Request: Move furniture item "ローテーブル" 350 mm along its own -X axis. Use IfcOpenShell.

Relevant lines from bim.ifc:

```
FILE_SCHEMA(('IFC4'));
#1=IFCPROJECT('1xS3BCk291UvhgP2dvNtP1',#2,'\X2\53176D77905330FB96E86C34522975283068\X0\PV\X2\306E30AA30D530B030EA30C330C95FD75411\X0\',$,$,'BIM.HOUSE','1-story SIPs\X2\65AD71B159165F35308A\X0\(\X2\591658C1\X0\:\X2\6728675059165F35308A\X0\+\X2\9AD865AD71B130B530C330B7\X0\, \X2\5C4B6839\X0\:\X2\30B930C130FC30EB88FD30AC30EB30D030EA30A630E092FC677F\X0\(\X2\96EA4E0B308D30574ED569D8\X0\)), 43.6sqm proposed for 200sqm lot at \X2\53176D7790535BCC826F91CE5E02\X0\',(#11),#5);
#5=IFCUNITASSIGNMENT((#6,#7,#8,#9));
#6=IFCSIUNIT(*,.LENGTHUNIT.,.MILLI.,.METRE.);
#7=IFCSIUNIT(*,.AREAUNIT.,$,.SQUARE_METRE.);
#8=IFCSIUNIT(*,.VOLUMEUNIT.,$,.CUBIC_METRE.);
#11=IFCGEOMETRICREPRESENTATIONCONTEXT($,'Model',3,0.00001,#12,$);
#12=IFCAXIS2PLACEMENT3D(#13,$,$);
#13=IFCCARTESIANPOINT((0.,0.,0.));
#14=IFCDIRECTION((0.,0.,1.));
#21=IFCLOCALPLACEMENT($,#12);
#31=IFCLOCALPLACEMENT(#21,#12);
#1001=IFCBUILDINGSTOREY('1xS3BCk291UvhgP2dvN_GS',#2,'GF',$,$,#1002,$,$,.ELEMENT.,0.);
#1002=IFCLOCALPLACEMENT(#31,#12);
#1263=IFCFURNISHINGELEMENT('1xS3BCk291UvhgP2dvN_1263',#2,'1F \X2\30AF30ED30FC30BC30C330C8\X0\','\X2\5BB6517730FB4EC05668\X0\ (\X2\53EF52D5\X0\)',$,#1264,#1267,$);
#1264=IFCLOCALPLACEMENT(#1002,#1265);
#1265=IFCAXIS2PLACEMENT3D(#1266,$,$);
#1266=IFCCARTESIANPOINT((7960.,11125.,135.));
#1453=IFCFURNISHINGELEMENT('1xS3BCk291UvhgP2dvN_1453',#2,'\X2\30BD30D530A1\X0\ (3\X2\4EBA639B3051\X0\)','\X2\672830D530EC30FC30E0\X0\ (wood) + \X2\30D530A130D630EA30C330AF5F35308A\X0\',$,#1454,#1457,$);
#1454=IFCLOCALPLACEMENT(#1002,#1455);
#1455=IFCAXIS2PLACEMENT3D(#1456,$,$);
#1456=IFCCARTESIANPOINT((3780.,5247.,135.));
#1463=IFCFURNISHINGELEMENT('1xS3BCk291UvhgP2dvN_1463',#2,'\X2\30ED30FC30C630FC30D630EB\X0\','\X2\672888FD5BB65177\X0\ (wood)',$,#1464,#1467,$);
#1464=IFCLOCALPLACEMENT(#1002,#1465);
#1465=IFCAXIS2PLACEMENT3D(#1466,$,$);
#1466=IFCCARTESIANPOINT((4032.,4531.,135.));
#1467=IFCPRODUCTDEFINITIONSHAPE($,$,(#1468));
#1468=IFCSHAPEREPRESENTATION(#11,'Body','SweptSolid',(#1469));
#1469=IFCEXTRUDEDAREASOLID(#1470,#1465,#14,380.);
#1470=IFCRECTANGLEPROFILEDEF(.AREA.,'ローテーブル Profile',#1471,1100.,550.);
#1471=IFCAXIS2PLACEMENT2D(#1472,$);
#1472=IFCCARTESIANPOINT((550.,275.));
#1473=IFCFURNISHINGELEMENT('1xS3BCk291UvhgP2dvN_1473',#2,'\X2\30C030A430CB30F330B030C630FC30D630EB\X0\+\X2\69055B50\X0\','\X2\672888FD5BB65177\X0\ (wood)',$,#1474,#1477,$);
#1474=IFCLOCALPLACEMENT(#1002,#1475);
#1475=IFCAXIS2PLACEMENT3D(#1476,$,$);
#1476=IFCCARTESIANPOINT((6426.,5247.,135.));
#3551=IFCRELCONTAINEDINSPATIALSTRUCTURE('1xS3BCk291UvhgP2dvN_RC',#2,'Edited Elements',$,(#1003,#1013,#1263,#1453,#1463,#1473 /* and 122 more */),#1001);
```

```python
import ifcopenshell
import ifcopenshell.api.geometry
import ifcopenshell.util.placement

model = ifcopenshell.open("bim.ifc")

item = model.by_guid("1xS3BCk291UvhgP2dvN_1463")
matrix = ifcopenshell.util.placement.get_local_placement(item.ObjectPlacement)
matrix[:3, 3] -= matrix[:3, 0] * 350.0
ifcopenshell.api.geometry.edit_object_placement(model, product=item, matrix=matrix, is_si=False)

print(ifcopenshell.util.placement.get_local_placement(item.ObjectPlacement).round(3) + 0.0)

model.write("bim_updated.ifc")
```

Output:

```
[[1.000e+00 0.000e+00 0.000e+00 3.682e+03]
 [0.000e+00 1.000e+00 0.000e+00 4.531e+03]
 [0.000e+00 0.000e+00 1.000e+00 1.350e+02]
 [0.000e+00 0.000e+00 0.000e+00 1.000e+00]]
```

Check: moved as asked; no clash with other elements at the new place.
